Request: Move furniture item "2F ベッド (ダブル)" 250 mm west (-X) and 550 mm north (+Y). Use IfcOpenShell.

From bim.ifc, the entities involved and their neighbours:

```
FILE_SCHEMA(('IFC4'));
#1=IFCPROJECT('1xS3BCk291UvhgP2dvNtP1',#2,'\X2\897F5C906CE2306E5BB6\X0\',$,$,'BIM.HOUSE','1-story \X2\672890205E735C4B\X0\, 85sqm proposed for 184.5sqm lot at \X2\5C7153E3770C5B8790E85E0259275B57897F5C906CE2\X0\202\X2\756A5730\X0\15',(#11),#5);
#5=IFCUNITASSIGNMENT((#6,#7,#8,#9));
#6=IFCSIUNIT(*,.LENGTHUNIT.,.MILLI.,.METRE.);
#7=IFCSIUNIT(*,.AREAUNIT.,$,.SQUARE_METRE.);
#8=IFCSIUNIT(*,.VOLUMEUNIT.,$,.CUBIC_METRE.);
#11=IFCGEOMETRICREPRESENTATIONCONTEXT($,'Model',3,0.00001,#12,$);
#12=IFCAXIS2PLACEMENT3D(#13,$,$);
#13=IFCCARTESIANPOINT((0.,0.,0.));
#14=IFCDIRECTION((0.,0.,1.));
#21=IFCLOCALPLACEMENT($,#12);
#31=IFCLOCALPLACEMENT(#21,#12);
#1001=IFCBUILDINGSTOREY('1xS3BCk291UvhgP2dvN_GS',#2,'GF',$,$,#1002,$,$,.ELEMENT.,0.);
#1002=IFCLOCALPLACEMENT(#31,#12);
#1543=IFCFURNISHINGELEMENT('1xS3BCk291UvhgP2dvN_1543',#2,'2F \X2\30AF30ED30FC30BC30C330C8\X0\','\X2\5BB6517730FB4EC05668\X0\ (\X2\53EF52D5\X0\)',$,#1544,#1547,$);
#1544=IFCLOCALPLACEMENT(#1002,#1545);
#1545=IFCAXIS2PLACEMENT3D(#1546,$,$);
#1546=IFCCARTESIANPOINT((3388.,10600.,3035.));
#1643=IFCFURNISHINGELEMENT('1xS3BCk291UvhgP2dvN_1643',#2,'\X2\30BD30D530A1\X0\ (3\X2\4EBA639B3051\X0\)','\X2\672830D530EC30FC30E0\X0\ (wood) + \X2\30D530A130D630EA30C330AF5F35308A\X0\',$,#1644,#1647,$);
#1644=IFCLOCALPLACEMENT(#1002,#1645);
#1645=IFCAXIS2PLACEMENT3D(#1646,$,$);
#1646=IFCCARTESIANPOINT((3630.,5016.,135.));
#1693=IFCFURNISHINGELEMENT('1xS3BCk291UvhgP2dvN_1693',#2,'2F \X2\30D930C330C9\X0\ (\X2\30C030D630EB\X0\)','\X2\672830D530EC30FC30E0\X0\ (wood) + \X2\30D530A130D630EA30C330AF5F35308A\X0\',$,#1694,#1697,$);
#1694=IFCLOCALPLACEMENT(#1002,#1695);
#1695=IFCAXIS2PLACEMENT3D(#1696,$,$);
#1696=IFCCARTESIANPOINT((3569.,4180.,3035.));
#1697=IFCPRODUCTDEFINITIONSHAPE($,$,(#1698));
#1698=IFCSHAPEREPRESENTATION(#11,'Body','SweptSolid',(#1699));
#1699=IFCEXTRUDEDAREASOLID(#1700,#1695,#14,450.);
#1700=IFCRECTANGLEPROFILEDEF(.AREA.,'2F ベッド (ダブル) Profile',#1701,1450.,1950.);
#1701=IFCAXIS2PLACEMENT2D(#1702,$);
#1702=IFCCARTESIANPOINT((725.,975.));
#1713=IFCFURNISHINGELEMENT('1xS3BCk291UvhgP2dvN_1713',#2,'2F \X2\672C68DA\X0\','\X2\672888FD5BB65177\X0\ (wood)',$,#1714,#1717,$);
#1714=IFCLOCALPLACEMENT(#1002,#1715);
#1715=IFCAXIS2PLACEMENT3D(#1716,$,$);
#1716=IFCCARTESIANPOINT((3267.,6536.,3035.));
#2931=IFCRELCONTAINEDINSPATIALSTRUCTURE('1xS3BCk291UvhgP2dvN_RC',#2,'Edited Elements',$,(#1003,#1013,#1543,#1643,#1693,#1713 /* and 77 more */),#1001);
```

```python
import ifcopenshell
import ifcopenshell.api.geometry
import ifcopenshell.util.placement
import ifcopenshell.util.unit

model = ifcopenshell.open("bim.ifc")
unit_scale = ifcopenshell.util.unit.calculate_unit_scale(model)

item = model.by_id(1693)
matrix = ifcopenshell.util.placement.get_local_placement(item.ObjectPlacement)
matrix[0, 3] -= 0.25 / unit_scale
matrix[1, 3] += 0.55 / unit_scale
ifcopenshell.api.geometry.edit_object_placement(model, product=item, matrix=matrix, is_si=False)

print(ifcopenshell.util.placement.get_local_placement(item.ObjectPlacement).round(3) + 0.0)

model.write("bim-out.ifc")
```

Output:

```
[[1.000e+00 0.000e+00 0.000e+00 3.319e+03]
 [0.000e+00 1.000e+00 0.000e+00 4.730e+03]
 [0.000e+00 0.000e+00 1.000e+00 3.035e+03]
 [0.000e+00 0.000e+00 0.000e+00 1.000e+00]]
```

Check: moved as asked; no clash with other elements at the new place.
